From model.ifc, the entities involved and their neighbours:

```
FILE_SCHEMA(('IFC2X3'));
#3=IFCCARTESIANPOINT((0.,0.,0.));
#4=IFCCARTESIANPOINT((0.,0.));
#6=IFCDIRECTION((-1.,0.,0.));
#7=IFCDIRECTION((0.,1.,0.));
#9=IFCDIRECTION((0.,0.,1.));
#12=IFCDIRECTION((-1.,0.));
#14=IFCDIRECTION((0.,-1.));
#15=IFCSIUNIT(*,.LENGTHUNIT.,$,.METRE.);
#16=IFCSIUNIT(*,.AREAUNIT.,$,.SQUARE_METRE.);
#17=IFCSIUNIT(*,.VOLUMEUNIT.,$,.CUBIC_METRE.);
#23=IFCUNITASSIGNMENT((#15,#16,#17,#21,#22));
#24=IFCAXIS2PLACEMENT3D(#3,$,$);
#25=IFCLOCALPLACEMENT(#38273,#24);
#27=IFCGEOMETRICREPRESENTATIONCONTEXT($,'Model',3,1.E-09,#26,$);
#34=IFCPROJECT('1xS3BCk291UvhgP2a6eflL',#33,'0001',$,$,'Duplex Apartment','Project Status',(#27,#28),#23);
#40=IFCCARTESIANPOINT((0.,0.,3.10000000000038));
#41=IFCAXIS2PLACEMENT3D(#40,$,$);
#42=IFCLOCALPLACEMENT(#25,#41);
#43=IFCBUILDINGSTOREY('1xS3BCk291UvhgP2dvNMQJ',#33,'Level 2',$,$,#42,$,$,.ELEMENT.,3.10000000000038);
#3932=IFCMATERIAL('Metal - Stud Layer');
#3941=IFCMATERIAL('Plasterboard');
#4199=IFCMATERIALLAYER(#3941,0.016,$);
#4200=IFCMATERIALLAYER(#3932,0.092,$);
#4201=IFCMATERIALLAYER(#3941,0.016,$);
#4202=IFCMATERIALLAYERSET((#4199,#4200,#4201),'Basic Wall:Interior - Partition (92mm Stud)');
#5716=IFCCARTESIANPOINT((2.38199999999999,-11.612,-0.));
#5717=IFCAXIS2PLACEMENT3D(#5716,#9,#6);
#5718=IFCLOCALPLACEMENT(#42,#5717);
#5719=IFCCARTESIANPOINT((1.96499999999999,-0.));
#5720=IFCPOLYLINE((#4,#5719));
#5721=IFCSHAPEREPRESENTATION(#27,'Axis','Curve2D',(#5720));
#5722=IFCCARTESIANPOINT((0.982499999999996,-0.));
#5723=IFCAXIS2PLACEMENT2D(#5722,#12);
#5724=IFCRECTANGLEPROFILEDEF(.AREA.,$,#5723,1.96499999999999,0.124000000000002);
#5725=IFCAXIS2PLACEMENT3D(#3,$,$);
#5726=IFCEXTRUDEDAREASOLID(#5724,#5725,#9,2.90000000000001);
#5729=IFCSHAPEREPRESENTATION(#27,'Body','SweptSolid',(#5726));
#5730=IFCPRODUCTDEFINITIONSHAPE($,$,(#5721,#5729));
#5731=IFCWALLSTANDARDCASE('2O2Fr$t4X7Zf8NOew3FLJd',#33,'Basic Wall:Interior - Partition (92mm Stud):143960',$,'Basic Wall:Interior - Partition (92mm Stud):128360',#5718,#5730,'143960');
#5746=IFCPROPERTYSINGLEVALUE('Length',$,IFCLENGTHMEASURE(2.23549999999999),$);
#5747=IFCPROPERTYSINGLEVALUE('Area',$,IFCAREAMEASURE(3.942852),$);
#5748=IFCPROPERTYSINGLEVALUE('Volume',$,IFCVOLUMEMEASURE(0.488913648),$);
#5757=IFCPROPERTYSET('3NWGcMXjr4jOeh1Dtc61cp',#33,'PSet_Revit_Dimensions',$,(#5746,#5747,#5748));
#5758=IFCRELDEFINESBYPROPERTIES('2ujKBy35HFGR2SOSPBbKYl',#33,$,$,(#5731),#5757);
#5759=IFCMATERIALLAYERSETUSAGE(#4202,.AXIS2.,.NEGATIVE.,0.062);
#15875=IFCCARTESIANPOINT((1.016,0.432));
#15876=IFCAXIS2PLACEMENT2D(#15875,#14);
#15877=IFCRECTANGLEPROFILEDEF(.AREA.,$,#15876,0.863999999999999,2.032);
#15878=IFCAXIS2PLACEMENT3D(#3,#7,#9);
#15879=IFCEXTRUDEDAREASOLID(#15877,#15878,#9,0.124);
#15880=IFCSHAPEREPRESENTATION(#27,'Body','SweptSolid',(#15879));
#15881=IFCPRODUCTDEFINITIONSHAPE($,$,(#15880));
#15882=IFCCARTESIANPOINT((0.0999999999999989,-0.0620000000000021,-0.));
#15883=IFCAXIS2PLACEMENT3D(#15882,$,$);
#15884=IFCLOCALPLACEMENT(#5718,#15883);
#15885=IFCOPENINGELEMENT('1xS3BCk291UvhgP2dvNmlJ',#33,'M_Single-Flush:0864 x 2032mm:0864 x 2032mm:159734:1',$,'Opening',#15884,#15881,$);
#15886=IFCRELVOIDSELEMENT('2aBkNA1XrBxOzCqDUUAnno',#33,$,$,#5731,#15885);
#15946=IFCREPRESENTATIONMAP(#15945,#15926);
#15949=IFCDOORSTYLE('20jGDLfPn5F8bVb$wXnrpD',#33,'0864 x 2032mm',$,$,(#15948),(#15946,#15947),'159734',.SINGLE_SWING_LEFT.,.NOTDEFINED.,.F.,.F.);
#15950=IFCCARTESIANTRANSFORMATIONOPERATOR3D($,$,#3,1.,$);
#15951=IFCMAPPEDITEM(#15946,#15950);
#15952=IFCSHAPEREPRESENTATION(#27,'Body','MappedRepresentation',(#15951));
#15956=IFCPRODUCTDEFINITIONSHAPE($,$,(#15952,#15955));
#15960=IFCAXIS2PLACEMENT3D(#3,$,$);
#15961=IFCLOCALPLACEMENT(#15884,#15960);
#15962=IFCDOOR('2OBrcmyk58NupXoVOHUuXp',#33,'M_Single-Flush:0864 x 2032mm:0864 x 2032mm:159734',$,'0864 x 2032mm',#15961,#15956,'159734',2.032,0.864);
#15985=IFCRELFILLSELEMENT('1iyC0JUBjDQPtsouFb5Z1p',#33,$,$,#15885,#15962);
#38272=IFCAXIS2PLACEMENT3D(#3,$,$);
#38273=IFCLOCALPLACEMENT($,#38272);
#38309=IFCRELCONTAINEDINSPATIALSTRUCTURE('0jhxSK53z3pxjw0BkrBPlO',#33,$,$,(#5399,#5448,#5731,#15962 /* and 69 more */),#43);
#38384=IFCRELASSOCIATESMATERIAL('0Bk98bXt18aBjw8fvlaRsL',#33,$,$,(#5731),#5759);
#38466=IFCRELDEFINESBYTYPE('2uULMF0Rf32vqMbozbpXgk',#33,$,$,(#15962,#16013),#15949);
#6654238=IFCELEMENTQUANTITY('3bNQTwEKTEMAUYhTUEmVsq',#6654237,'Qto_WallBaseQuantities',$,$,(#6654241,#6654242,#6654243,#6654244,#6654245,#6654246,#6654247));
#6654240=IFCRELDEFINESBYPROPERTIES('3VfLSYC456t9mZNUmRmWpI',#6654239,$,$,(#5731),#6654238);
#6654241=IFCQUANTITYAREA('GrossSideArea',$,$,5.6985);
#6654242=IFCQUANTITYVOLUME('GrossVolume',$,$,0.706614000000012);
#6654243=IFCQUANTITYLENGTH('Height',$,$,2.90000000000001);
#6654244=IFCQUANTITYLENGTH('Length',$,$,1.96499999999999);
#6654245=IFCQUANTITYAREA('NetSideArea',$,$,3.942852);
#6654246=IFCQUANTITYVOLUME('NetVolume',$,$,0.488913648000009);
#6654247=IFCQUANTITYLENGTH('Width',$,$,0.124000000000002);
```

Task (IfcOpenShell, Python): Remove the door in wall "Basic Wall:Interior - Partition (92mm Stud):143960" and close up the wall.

```python
import ifcopenshell
import ifcopenshell.api.feature
import ifcopenshell.api.pset
import ifcopenshell.api.root
import ifcopenshell.geom
import ifcopenshell.util.element
import ifcopenshell.util.shape
import ifcopenshell.util.unit

model = ifcopenshell.open("model.ifc")
area_scale = ifcopenshell.util.unit.calculate_unit_scale(model, "AREAUNIT")
volume_scale = ifcopenshell.util.unit.calculate_unit_scale(model, "VOLUMEUNIT")
settings = ifcopenshell.geom.settings()


def volume(element):
    """Net volume in cubic metres, openings subtracted."""
    shape = ifcopenshell.geom.create_shape(settings, element)
    return ifcopenshell.util.shape.get_volume(shape.geometry)


door = model.by_guid("2OBrcmyk58NupXoVOHUuXp")
opening = door.FillsVoids[0].RelatingOpeningElement
wall = opening.VoidsElements[0].RelatingBuildingElement
before = volume(wall)

ifcopenshell.api.root.remove_product(model, product=door)
ifcopenshell.api.feature.remove_feature(model, feature=opening)

after = volume(wall)
thickness = 0.124  # wall thickness in metres

# Update the wall's stored quantities.
pset = model.by_id(ifcopenshell.util.element.get_pset(wall, "PSet_Revit_Dimensions", should_inherit=False)["id"])
ifcopenshell.api.pset.edit_pset(model, pset=pset, properties={
    "Area": model.create_entity("IfcAreaMeasure", after / thickness / area_scale),
    "Volume": model.create_entity("IfcVolumeMeasure", after / volume_scale),
})
qto = model.by_id(ifcopenshell.util.element.get_pset(wall, "Qto_WallBaseQuantities", should_inherit=False)["id"])
ifcopenshell.api.pset.edit_qto(model, qto=qto, properties={
    "NetSideArea": after / thickness / area_scale,
    "NetVolume": after / volume_scale,
})

print(f"wall volume {before:.3f} -> {after:.3f} m3")

model.write("model_v2.ifc")
```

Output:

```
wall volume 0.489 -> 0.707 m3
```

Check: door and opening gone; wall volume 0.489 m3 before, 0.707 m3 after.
